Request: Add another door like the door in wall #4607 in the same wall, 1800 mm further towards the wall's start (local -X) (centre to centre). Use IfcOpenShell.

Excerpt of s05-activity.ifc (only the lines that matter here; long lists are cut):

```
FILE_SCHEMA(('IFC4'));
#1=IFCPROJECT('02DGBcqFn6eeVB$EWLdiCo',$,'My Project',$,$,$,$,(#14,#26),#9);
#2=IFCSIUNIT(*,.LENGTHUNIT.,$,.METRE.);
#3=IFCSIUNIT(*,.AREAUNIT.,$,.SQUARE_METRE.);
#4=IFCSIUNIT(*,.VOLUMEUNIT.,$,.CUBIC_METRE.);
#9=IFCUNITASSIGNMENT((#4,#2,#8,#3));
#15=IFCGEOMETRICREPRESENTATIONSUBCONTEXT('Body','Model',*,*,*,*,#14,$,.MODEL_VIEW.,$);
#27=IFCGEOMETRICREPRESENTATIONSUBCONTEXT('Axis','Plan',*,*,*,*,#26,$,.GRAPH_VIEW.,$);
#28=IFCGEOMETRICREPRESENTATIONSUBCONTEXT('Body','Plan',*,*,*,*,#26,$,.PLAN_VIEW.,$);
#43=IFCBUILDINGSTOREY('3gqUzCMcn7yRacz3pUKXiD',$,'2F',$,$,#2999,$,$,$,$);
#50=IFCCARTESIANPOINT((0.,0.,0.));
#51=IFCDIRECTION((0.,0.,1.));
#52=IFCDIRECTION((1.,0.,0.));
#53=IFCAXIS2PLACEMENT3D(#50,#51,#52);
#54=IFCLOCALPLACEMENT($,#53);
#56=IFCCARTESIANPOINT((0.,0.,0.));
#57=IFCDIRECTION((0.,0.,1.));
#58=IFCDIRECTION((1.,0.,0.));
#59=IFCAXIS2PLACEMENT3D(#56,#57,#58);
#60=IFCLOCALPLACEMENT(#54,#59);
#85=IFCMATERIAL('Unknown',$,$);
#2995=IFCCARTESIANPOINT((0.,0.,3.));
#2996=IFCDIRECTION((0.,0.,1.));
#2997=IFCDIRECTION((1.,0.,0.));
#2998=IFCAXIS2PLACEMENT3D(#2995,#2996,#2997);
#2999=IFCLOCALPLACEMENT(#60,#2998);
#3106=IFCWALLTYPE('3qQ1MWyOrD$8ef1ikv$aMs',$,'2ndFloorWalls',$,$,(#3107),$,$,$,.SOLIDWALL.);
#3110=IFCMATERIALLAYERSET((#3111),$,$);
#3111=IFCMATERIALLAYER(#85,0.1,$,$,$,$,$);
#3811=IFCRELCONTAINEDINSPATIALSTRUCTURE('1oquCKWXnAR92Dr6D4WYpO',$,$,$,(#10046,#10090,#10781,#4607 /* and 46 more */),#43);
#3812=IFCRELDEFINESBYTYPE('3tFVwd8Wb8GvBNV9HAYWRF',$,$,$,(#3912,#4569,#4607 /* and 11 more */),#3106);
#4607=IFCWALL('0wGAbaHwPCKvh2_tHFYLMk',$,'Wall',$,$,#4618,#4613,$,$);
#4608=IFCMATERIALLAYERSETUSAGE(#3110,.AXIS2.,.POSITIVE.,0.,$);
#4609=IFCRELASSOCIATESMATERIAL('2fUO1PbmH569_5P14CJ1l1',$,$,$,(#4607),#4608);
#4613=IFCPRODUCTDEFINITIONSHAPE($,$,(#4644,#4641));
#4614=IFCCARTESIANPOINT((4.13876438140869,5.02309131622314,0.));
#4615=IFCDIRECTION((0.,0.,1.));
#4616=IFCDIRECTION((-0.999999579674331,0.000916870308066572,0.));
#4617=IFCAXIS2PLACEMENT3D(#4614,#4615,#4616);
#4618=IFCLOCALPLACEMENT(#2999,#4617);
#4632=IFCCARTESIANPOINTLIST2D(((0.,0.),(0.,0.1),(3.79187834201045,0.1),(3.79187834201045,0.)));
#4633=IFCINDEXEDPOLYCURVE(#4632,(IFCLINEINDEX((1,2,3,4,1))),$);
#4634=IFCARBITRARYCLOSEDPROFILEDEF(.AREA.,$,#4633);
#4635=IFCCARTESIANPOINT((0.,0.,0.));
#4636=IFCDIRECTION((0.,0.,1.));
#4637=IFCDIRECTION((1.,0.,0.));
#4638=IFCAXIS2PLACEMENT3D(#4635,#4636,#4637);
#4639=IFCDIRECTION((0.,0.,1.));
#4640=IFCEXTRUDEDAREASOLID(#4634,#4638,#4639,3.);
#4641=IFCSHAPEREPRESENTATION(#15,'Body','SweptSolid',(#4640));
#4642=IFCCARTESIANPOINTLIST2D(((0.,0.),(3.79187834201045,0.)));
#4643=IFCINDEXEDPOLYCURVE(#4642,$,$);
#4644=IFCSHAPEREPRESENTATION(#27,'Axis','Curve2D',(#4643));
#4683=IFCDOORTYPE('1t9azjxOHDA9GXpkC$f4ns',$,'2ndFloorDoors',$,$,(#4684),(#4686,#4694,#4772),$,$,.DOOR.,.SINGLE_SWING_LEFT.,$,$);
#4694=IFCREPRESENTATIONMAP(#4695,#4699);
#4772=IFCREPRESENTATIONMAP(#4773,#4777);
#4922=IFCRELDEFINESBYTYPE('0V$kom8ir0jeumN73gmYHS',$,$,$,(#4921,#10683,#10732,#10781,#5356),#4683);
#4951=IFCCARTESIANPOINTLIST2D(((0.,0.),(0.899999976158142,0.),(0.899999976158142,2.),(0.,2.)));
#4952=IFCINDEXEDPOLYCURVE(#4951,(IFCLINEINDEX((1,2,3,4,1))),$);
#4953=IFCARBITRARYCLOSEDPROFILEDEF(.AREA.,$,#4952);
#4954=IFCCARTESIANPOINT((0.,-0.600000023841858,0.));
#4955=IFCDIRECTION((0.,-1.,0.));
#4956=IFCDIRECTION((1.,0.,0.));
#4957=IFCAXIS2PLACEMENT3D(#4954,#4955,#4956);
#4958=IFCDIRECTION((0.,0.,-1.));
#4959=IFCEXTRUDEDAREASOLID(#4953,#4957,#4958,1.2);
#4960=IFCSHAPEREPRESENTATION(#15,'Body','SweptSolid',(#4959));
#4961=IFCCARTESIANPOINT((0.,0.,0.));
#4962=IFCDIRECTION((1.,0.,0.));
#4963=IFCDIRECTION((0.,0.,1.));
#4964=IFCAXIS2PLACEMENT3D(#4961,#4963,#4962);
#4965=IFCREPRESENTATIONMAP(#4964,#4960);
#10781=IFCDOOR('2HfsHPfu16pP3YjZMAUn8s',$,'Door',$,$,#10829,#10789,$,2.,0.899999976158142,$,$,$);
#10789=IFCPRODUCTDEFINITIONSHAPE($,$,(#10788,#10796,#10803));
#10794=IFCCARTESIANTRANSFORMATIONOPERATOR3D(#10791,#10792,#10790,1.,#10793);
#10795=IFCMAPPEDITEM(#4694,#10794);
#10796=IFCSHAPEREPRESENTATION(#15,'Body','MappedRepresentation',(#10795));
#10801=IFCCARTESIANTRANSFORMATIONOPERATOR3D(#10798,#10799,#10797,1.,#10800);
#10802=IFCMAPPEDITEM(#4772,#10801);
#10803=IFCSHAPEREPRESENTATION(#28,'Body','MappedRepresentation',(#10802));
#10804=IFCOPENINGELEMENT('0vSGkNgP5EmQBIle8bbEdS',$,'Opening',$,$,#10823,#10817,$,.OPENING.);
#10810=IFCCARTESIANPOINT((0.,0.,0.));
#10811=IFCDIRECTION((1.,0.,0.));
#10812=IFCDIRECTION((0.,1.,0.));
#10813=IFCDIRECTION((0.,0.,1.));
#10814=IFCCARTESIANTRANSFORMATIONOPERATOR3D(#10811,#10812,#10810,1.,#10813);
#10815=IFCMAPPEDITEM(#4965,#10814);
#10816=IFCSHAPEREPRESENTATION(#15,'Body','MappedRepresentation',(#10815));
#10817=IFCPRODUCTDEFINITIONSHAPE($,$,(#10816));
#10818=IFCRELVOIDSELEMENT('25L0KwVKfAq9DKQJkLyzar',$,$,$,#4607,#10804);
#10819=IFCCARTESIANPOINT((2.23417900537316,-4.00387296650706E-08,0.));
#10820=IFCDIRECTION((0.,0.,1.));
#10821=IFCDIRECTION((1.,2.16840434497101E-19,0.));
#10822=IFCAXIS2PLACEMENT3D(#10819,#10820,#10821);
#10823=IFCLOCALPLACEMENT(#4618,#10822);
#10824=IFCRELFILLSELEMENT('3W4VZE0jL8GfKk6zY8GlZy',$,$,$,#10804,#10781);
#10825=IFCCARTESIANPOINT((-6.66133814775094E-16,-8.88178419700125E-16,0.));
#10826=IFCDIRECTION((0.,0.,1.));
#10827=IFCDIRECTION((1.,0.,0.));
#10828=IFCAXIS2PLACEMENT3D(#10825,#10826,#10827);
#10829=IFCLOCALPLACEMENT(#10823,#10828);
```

```python
import ifcopenshell
import ifcopenshell.api.feature
import ifcopenshell.api.geometry
import ifcopenshell.api.root
import ifcopenshell.geom
import ifcopenshell.util.element
import ifcopenshell.util.placement
import ifcopenshell.util.shape

model = ifcopenshell.open("s05-activity.ifc")
settings = ifcopenshell.geom.settings()


def volume(element):
    """Net volume in cubic metres, openings subtracted."""
    shape = ifcopenshell.geom.create_shape(settings, element)
    return ifcopenshell.util.shape.get_volume(shape.geometry)


door = model.by_guid("2HfsHPfu16pP3YjZMAUn8s")
opening = door.FillsVoids[0].RelatingOpeningElement
wall = opening.VoidsElements[0].RelatingBuildingElement
before = volume(wall)
shift = ifcopenshell.util.placement.get_local_placement(wall.ObjectPlacement)[:3, 0] * -1.8

# copy_class copies the void relationship, type, container and properties, but no geometry.
new_opening = ifcopenshell.api.root.copy_class(model, product=opening)
new_opening.Representation = ifcopenshell.util.element.copy_deep(
    model, opening.Representation, exclude=["IfcGeometricRepresentationContext", "IfcRepresentationMap"]
)
new_door = ifcopenshell.api.root.copy_class(model, product=door)
new_door.Representation = ifcopenshell.util.element.copy_deep(
    model, door.Representation, exclude=["IfcGeometricRepresentationContext", "IfcRepresentationMap"]
)
ifcopenshell.api.feature.add_filling(model, opening=new_opening, element=new_door)

for old, new in ((opening, new_opening), (door, new_door)):
    matrix = ifcopenshell.util.placement.get_local_placement(old.ObjectPlacement)
    matrix[:3, 3] += shift
    ifcopenshell.api.geometry.edit_object_placement(model, product=new, matrix=matrix, is_si=False)

after = volume(wall)

print(f"wall volume {before:.3f} -> {after:.3f} m3")

model.write("s05-activity_rev.ifc")
```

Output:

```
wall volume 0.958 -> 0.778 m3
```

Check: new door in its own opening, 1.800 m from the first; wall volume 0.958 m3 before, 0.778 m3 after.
